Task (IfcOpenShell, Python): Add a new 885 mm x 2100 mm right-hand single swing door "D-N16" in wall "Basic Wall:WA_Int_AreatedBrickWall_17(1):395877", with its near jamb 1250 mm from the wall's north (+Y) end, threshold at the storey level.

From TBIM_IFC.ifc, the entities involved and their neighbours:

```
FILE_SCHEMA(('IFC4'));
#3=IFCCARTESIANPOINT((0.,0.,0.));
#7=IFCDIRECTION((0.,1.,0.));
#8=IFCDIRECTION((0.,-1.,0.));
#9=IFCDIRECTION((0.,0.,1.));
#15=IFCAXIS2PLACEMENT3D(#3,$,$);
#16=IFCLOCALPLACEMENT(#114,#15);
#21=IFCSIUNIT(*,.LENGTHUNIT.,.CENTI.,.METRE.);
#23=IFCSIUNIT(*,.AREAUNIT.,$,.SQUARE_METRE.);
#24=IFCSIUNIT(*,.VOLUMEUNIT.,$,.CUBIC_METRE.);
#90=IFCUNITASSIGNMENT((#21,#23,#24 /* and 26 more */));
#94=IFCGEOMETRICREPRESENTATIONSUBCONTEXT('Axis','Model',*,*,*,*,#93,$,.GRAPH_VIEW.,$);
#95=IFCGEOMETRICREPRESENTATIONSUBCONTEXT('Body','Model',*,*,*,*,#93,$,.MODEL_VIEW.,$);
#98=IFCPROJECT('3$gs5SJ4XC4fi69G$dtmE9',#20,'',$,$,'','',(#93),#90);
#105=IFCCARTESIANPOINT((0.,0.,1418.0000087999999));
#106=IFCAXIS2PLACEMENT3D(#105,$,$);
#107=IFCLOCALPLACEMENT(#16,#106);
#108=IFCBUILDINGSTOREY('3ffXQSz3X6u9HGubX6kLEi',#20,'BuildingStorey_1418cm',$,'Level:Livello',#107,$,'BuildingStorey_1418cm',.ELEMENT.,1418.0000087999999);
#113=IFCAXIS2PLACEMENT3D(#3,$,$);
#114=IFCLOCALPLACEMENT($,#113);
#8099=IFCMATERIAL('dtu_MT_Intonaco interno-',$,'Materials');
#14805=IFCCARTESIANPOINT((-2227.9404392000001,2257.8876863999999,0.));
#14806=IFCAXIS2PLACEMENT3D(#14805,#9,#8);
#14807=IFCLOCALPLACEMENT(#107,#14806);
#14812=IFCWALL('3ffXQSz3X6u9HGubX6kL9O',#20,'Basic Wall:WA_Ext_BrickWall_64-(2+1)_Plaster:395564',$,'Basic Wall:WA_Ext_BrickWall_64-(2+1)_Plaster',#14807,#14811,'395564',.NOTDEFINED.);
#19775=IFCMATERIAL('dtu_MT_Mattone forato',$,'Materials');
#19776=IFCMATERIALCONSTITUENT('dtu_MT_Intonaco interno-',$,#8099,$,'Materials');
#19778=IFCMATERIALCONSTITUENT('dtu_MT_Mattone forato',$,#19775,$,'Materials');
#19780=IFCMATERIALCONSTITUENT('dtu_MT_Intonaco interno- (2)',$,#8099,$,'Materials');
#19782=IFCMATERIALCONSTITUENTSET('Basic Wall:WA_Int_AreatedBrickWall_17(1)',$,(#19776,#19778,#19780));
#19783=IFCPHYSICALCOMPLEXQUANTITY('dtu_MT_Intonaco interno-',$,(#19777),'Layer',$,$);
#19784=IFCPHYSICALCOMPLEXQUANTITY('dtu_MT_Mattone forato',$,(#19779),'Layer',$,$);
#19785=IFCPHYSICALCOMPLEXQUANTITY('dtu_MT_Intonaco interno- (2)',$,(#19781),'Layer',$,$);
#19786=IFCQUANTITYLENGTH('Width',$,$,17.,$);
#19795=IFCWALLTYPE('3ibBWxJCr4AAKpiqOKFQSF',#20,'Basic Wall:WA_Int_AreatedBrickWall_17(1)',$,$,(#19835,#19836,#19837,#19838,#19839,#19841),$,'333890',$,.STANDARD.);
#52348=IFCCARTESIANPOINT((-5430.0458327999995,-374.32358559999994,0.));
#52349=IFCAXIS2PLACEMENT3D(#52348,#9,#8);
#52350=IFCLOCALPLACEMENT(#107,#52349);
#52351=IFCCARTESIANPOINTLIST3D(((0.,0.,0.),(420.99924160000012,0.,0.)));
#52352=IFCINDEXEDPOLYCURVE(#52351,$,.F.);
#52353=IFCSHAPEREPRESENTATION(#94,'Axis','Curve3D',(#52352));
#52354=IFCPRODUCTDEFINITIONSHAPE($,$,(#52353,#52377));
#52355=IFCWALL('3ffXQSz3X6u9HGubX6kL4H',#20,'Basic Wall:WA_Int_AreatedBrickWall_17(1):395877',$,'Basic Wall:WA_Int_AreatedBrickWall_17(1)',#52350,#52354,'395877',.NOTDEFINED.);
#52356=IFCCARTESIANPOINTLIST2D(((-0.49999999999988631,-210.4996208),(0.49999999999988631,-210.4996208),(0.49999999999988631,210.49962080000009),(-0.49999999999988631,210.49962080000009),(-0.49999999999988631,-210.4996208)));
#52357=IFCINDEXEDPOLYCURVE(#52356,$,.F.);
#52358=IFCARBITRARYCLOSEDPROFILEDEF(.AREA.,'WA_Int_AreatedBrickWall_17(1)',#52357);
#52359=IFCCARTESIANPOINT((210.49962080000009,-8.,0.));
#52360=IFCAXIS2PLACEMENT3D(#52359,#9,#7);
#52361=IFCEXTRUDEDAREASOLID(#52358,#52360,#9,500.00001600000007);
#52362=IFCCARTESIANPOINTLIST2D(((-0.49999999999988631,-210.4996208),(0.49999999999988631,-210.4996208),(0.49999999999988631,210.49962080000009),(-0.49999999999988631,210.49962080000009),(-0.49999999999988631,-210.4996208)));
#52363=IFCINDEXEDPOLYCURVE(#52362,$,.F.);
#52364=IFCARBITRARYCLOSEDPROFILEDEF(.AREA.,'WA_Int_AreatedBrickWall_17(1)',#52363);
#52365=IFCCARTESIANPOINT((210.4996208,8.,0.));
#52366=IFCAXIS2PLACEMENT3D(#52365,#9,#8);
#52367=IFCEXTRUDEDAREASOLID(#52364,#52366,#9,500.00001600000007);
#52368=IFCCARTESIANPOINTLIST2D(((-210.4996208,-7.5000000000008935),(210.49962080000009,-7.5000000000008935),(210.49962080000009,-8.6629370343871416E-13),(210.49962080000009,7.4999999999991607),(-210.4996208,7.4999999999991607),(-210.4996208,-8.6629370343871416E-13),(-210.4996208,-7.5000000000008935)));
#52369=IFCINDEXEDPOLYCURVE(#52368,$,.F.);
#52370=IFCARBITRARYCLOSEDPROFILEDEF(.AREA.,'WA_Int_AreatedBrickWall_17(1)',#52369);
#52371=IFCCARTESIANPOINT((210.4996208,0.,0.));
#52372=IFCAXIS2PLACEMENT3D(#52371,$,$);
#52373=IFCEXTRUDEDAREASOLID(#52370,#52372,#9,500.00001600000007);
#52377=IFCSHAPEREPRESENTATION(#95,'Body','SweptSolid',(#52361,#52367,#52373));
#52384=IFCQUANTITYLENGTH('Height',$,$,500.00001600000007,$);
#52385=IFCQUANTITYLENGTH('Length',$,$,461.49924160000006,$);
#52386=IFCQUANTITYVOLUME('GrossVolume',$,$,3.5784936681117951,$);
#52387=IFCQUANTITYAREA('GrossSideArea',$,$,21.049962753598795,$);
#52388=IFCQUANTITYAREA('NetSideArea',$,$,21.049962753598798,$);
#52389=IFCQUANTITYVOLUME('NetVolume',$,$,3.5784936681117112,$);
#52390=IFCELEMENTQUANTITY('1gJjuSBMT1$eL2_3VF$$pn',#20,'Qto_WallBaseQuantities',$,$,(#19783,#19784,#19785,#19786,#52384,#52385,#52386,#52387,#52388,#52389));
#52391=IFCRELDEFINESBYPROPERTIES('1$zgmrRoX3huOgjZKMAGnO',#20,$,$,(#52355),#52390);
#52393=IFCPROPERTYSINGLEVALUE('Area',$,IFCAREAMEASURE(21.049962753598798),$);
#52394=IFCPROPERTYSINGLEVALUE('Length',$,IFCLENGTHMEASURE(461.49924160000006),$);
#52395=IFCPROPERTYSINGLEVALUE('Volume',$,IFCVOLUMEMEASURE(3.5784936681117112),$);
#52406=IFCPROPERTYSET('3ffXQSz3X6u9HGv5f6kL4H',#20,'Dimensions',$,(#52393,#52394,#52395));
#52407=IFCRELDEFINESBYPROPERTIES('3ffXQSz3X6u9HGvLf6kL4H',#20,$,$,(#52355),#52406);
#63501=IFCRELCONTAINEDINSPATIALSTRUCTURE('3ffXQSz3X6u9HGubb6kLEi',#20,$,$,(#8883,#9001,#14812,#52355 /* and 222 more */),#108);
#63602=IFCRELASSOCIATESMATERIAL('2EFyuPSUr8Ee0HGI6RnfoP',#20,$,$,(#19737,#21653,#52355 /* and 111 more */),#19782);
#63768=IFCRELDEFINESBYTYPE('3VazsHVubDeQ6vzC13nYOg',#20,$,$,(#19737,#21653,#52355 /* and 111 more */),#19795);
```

```python
import numpy as np
import ifcopenshell
import ifcopenshell.api.feature
import ifcopenshell.api.geometry
import ifcopenshell.api.pset
import ifcopenshell.api.root
import ifcopenshell.api.spatial
import ifcopenshell.geom
import ifcopenshell.util.element
import ifcopenshell.util.placement
import ifcopenshell.util.representation
import ifcopenshell.util.shape
import ifcopenshell.util.unit

model = ifcopenshell.open("TBIM_IFC.ifc")
unit_scale = ifcopenshell.util.unit.calculate_unit_scale(model)
area_scale = ifcopenshell.util.unit.calculate_unit_scale(model, "AREAUNIT")
volume_scale = ifcopenshell.util.unit.calculate_unit_scale(model, "VOLUMEUNIT")
settings = ifcopenshell.geom.settings()


def volume(element):
    """Net volume in cubic metres, openings subtracted."""
    shape = ifcopenshell.geom.create_shape(settings, element)
    return ifcopenshell.util.shape.get_volume(shape.geometry)


wall = model.by_guid("3ffXQSz3X6u9HGubX6kL4H")
storey = ifcopenshell.util.element.get_container(wall, ifc_class="IfcBuildingStorey")
context = ifcopenshell.util.representation.get_context(model, "Model", "Body", "MODEL_VIEW")
before = volume(wall)

width, height, from_end, sill = 0.885, 2.1, 1.25, 0.0  # metres

# The wall runs along its own X axis, and the end named is its -X end.
wall_shape = ifcopenshell.geom.create_shape(settings, wall)
x, y, z = ifcopenshell.util.shape.get_vertices(wall_shape.geometry).T
start = x.min() + from_end
face, thickness = float(y.min()), float(y.max() - y.min())
wall_matrix = ifcopenshell.util.placement.get_local_placement(wall.ObjectPlacement)
level = ifcopenshell.util.placement.get_local_placement(storey.ObjectPlacement)[2, 3]


def in_wall(x, y):
    """Placement at x, y metres in the wall's axes, at sill height."""
    matrix = wall_matrix.copy()
    matrix[:, 3] = wall_matrix @ np.array([x / unit_scale, y / unit_scale, 0.0, 1.0])
    matrix[2, 3] = level + sill / unit_scale
    return matrix


# Opening: a box that overshoots both wall faces by 50 mm.
opening = ifcopenshell.api.root.create_entity(model, ifc_class="IfcOpeningElement", predefined_type="OPENING")
box = ifcopenshell.api.geometry.add_wall_representation(
    model, context=context, length=width, height=height, thickness=thickness + 0.1
)
ifcopenshell.api.geometry.assign_representation(model, product=opening, representation=box)
ifcopenshell.api.geometry.edit_object_placement(model, product=opening, matrix=in_wall(start, face - 0.05), is_si=False)
ifcopenshell.api.feature.add_feature(model, feature=opening, element=wall)

door = ifcopenshell.api.root.create_entity(model, ifc_class="IfcDoor", name="D-N16", predefined_type="DOOR")
door.OverallWidth, door.OverallHeight = width / unit_scale, height / unit_scale
door.OperationType = "SINGLE_SWING_RIGHT"
body = ifcopenshell.api.geometry.add_door_representation(
    model,
    context=context,
    overall_width=door.OverallWidth,
    overall_height=door.OverallHeight,
    operation_type="SINGLE_SWING_RIGHT",
    lining_properties={"LiningDepth": thickness / unit_scale, "ThresholdDepth": thickness / unit_scale},
)
ifcopenshell.api.geometry.assign_representation(model, product=door, representation=body)
ifcopenshell.api.spatial.assign_container(model, products=[door], relating_structure=storey)
ifcopenshell.api.feature.add_filling(model, opening=opening, element=door)

# The lining spans the wall, so the door starts at the wall face.
ifcopenshell.api.geometry.edit_object_placement(model, product=door, matrix=in_wall(start, face), is_si=False)

after = volume(wall)

# Update the wall's stored quantities.
qto = model.by_id(ifcopenshell.util.element.get_pset(wall, "Qto_WallBaseQuantities", should_inherit=False)["id"])
ifcopenshell.api.pset.edit_qto(model, qto=qto, properties={
    "NetSideArea": after / thickness / area_scale,
    "NetVolume": after / volume_scale,
})
pset = model.by_id(ifcopenshell.util.element.get_pset(wall, "Dimensions", should_inherit=False)["id"])
ifcopenshell.api.pset.edit_pset(model, pset=pset, properties={
    "Area": model.create_entity("IfcAreaMeasure", after / thickness / area_scale),
    "Volume": model.create_entity("IfcVolumeMeasure", after / volume_scale),
})

print(f"wall volume {before:.3f} -> {after:.3f} m3")

model.write("TBIM_IFC_v2.ifc")
```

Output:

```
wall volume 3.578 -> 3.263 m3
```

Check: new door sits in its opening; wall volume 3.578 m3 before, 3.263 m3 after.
